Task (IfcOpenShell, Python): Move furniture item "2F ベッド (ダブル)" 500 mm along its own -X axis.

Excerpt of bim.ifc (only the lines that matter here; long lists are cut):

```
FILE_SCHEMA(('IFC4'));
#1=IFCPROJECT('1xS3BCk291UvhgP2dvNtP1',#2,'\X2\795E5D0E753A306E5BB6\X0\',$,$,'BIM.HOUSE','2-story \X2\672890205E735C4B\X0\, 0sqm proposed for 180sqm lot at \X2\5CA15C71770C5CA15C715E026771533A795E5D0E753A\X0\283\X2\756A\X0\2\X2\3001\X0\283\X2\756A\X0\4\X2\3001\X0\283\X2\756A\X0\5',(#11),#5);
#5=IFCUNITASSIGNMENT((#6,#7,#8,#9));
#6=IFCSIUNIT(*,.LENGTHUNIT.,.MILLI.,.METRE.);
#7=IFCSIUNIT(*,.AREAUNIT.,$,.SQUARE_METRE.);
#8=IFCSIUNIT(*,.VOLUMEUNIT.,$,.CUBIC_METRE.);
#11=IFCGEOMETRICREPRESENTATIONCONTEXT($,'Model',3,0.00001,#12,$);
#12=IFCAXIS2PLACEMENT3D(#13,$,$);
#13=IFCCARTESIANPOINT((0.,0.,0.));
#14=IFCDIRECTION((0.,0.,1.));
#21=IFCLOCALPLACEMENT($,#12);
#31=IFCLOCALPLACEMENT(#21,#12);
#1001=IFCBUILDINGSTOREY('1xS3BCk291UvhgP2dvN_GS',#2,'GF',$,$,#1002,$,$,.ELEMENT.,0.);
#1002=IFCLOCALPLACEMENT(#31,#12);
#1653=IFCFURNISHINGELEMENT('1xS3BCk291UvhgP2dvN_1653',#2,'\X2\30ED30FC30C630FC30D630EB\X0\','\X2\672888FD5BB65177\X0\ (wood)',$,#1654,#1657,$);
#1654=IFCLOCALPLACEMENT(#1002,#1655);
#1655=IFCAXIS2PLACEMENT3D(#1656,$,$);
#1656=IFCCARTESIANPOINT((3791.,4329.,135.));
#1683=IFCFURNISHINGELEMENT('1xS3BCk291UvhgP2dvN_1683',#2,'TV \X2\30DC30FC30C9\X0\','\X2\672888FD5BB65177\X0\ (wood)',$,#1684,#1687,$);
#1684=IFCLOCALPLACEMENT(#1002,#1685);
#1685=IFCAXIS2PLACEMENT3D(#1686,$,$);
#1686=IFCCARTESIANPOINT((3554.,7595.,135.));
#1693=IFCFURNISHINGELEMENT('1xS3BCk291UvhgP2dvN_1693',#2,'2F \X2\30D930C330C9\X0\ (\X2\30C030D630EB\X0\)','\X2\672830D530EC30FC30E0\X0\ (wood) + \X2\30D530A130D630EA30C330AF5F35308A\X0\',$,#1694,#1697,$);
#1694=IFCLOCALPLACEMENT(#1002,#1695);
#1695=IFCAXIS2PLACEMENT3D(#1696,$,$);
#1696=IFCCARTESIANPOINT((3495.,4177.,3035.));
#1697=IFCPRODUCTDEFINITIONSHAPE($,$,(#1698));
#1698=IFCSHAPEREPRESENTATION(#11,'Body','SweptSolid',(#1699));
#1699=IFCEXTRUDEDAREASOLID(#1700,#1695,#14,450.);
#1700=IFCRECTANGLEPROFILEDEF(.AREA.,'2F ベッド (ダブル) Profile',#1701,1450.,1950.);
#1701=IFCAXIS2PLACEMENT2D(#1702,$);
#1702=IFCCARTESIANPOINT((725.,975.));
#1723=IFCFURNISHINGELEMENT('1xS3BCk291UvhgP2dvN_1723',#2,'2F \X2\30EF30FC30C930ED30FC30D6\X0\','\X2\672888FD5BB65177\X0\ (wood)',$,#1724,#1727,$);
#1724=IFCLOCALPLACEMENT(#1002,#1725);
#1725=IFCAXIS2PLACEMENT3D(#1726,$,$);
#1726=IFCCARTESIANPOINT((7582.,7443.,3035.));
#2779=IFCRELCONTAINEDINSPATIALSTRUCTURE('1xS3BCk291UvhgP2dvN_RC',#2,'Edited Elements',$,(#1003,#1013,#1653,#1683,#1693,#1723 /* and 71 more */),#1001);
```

```python
import ifcopenshell
import ifcopenshell.api.geometry
import ifcopenshell.util.placement
import ifcopenshell.util.unit

model = ifcopenshell.open("bim.ifc")
unit_scale = ifcopenshell.util.unit.calculate_unit_scale(model)

item = model.by_guid("1xS3BCk291UvhgP2dvN_1693")
matrix = ifcopenshell.util.placement.get_local_placement(item.ObjectPlacement)
matrix[:3, 3] -= matrix[:3, 0] * 0.5 / unit_scale
ifcopenshell.api.geometry.edit_object_placement(model, product=item, matrix=matrix, is_si=False)

print(ifcopenshell.util.placement.get_local_placement(item.ObjectPlacement).round(3) + 0.0)

model.write("bim-out.ifc")
```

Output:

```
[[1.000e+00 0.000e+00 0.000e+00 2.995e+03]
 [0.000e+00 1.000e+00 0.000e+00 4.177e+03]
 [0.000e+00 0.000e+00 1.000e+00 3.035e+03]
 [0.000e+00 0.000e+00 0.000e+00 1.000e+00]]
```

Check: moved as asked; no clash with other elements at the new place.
